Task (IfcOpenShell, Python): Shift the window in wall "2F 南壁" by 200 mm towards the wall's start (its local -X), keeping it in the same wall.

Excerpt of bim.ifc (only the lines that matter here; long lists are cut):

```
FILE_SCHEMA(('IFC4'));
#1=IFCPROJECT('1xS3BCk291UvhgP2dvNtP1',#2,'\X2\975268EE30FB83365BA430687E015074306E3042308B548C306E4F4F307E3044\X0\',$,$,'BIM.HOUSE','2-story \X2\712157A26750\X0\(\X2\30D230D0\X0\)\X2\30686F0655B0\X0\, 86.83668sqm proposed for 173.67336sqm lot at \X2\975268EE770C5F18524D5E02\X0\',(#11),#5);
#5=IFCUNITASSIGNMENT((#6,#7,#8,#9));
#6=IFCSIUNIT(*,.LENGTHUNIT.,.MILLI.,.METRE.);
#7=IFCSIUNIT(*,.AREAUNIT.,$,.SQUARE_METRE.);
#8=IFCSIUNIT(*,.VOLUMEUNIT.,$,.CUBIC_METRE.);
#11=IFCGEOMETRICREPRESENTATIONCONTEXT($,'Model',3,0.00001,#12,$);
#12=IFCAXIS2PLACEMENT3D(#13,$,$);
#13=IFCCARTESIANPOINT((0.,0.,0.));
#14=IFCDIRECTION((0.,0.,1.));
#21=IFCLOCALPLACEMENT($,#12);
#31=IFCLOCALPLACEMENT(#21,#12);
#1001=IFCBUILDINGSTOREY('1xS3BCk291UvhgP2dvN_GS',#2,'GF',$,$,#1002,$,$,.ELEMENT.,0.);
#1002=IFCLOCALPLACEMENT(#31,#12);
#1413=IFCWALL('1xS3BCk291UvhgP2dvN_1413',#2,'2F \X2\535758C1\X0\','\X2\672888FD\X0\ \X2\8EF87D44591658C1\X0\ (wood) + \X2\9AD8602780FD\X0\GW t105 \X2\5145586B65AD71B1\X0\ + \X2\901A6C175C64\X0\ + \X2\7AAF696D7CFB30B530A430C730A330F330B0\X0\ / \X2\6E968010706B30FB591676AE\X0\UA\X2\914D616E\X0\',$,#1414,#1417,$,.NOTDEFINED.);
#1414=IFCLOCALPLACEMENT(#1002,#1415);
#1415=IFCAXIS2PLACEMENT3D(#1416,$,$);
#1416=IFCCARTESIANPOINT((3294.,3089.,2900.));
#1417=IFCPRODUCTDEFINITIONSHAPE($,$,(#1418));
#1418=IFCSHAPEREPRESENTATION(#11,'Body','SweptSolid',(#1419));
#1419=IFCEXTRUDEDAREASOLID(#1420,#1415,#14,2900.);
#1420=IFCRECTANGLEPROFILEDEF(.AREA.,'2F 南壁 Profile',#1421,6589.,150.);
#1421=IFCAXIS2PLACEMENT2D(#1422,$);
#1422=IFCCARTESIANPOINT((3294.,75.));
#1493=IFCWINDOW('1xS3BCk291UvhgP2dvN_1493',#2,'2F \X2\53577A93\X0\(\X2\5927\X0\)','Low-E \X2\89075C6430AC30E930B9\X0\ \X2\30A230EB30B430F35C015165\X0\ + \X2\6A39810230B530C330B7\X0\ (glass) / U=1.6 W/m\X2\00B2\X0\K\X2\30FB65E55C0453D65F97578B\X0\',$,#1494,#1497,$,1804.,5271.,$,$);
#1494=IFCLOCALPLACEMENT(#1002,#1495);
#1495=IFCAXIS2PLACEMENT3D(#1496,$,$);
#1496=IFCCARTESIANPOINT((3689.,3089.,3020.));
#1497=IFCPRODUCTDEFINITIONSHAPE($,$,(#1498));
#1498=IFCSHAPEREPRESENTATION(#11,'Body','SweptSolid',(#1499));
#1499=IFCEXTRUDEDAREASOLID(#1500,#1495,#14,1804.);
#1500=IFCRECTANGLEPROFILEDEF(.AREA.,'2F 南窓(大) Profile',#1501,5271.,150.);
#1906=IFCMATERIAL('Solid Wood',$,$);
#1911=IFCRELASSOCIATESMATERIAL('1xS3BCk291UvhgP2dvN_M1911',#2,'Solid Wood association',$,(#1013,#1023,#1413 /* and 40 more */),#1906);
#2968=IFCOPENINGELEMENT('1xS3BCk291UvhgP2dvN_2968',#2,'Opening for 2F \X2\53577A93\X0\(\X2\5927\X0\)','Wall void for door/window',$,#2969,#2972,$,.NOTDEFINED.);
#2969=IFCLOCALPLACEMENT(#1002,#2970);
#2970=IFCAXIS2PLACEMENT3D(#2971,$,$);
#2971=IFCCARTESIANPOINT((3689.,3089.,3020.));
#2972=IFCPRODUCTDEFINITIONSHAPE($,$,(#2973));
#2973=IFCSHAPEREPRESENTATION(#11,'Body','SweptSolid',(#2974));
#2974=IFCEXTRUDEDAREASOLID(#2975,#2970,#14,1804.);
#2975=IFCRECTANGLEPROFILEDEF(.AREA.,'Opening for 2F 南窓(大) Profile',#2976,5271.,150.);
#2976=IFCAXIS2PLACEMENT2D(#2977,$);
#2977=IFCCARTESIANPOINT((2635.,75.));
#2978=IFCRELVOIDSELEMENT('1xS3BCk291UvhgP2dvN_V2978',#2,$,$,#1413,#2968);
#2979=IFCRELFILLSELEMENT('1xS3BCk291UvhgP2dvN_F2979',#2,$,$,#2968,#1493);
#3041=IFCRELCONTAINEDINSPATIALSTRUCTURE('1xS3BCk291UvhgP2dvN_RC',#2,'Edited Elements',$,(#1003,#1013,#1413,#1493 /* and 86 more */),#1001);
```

```python
import ifcopenshell
import ifcopenshell.api.geometry
import ifcopenshell.util.placement
import ifcopenshell.util.unit

model = ifcopenshell.open("bim.ifc")
unit_scale = ifcopenshell.util.unit.calculate_unit_scale(model)

window = model.by_id(1493)
opening = window.FillsVoids[0].RelatingOpeningElement
wall = opening.VoidsElements[0].RelatingBuildingElement

wall_matrix = ifcopenshell.util.placement.get_local_placement(wall.ObjectPlacement)
shift = wall_matrix[:3, 0] * -0.2 / unit_scale
before = ifcopenshell.util.placement.get_local_placement(window.ObjectPlacement)[:3, 3].copy()

# The window is not placed relative to its opening, so move both.
for product in (opening, window):
    matrix = ifcopenshell.util.placement.get_local_placement(product.ObjectPlacement)
    matrix[:3, 3] += shift
    ifcopenshell.api.geometry.edit_object_placement(model, product=product, matrix=matrix, is_si=False)

after = ifcopenshell.util.placement.get_local_placement(window.ObjectPlacement)[:3, 3]
print("window moved by", (after - before).round(3) + 0.0)

model.write("bim_updated.ifc")
```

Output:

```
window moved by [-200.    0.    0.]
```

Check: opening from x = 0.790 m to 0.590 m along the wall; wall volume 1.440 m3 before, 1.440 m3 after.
